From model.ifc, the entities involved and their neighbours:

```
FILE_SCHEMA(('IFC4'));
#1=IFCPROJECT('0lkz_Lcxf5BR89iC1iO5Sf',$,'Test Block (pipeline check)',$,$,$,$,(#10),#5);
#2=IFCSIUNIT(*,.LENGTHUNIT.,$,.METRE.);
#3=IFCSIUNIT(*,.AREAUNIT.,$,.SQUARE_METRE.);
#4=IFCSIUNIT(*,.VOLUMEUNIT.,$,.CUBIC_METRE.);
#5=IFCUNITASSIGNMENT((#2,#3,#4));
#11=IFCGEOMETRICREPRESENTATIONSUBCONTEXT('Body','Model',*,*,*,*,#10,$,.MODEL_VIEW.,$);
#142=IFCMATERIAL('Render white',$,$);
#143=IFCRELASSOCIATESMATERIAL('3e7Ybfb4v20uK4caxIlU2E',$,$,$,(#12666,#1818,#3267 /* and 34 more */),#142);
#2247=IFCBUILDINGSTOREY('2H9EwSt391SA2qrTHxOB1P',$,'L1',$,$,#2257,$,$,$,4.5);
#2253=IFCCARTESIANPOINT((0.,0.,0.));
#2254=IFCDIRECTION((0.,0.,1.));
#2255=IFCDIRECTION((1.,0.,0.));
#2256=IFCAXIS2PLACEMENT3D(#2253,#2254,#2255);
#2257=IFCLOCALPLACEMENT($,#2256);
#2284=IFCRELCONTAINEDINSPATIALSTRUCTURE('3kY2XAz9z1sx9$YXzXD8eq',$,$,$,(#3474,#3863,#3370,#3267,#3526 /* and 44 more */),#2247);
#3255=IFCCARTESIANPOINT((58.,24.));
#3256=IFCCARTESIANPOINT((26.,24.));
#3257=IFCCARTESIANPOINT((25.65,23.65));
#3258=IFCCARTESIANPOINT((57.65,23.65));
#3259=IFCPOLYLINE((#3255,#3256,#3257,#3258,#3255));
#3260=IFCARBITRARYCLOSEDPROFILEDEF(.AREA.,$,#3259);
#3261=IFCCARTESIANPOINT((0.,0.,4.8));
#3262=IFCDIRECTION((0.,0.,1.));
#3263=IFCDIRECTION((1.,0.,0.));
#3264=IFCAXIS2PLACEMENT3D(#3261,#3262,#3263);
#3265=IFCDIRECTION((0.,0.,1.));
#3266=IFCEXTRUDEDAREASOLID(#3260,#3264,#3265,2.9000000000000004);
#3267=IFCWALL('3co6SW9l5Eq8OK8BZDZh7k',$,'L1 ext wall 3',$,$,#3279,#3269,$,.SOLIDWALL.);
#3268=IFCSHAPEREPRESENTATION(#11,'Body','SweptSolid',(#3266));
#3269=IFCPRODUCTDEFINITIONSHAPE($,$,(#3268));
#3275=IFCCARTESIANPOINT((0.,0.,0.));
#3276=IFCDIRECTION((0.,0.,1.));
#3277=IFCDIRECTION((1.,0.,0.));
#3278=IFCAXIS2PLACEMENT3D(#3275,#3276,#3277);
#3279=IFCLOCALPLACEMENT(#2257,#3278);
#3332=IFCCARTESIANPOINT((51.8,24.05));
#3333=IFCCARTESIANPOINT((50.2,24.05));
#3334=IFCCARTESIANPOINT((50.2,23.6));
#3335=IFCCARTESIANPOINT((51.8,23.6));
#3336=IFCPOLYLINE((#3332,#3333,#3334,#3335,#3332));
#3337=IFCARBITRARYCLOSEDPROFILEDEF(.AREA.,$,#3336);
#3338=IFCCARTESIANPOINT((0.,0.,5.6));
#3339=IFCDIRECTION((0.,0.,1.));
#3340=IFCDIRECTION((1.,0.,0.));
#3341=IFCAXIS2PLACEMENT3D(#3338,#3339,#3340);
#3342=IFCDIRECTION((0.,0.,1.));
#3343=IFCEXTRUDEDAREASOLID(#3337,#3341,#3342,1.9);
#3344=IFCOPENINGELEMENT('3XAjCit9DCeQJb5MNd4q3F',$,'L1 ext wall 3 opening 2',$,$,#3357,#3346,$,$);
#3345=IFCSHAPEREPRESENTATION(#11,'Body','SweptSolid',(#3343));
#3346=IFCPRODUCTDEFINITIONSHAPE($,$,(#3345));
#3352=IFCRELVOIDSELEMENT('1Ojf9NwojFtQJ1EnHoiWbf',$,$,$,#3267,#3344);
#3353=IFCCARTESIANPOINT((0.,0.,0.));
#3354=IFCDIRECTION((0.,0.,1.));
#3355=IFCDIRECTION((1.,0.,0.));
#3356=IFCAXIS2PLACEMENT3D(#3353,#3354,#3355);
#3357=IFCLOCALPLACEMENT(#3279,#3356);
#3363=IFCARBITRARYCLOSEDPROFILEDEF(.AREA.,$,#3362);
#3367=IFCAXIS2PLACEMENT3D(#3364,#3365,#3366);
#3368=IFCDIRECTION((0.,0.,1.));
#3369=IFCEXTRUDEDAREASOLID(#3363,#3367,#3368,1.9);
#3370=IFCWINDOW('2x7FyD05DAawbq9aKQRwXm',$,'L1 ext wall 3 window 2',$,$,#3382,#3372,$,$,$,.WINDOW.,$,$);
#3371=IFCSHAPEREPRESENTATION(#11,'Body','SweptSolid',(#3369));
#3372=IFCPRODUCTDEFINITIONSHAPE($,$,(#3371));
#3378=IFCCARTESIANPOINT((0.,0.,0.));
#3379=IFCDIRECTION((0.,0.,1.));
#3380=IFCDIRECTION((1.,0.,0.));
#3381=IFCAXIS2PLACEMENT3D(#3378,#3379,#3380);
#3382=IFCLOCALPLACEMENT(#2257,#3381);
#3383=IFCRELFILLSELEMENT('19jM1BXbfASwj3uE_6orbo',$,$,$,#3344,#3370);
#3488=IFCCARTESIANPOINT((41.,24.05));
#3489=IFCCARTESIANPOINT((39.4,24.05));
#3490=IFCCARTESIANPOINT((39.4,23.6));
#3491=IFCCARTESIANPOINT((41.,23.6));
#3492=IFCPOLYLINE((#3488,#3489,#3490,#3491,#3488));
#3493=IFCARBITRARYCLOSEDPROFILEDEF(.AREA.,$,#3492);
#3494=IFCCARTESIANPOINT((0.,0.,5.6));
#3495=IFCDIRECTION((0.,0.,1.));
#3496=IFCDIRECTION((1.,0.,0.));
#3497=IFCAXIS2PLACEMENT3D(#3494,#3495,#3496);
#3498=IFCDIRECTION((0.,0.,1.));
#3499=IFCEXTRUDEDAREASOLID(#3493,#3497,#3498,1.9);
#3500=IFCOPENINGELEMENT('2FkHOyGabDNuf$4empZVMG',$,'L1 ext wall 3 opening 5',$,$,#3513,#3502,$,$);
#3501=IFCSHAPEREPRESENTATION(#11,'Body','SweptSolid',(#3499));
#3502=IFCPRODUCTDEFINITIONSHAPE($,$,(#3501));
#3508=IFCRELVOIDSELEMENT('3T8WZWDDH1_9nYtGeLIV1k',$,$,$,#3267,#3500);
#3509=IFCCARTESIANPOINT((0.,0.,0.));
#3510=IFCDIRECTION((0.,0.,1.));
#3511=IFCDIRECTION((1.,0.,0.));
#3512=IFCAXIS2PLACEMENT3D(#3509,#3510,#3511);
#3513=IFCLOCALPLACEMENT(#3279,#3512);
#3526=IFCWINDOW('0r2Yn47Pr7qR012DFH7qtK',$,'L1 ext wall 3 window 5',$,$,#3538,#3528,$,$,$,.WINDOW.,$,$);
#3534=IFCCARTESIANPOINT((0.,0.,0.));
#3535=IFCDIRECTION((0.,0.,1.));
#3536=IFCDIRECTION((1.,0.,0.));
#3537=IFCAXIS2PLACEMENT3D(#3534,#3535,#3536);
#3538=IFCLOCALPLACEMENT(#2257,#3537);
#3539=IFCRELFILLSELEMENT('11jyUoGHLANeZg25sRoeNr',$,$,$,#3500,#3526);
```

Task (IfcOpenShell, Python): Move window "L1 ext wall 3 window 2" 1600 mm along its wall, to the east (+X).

```python
import ifcopenshell
import ifcopenshell.api.geometry
import ifcopenshell.util.placement

model = ifcopenshell.open("model.ifc")

window = model.by_guid("2x7FyD05DAawbq9aKQRwXm")
opening = window.FillsVoids[0].RelatingOpeningElement
wall = opening.VoidsElements[0].RelatingBuildingElement

wall_matrix = ifcopenshell.util.placement.get_local_placement(wall.ObjectPlacement)
shift = wall_matrix[:3, 0] * 1.6
before = ifcopenshell.util.placement.get_local_placement(window.ObjectPlacement)[:3, 3].copy()

# The window is not placed relative to its opening, so move both.
for product in (opening, window):
    matrix = ifcopenshell.util.placement.get_local_placement(product.ObjectPlacement)
    matrix[:3, 3] += shift
    ifcopenshell.api.geometry.edit_object_placement(model, product=product, matrix=matrix, is_si=False)

after = ifcopenshell.util.placement.get_local_placement(window.ObjectPlacement)[:3, 3]
print("window moved by", (after - before).round(3) + 0.0)

model.write("model_updated.ifc")
```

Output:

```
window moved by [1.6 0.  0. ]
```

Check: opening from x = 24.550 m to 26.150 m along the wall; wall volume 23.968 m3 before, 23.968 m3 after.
